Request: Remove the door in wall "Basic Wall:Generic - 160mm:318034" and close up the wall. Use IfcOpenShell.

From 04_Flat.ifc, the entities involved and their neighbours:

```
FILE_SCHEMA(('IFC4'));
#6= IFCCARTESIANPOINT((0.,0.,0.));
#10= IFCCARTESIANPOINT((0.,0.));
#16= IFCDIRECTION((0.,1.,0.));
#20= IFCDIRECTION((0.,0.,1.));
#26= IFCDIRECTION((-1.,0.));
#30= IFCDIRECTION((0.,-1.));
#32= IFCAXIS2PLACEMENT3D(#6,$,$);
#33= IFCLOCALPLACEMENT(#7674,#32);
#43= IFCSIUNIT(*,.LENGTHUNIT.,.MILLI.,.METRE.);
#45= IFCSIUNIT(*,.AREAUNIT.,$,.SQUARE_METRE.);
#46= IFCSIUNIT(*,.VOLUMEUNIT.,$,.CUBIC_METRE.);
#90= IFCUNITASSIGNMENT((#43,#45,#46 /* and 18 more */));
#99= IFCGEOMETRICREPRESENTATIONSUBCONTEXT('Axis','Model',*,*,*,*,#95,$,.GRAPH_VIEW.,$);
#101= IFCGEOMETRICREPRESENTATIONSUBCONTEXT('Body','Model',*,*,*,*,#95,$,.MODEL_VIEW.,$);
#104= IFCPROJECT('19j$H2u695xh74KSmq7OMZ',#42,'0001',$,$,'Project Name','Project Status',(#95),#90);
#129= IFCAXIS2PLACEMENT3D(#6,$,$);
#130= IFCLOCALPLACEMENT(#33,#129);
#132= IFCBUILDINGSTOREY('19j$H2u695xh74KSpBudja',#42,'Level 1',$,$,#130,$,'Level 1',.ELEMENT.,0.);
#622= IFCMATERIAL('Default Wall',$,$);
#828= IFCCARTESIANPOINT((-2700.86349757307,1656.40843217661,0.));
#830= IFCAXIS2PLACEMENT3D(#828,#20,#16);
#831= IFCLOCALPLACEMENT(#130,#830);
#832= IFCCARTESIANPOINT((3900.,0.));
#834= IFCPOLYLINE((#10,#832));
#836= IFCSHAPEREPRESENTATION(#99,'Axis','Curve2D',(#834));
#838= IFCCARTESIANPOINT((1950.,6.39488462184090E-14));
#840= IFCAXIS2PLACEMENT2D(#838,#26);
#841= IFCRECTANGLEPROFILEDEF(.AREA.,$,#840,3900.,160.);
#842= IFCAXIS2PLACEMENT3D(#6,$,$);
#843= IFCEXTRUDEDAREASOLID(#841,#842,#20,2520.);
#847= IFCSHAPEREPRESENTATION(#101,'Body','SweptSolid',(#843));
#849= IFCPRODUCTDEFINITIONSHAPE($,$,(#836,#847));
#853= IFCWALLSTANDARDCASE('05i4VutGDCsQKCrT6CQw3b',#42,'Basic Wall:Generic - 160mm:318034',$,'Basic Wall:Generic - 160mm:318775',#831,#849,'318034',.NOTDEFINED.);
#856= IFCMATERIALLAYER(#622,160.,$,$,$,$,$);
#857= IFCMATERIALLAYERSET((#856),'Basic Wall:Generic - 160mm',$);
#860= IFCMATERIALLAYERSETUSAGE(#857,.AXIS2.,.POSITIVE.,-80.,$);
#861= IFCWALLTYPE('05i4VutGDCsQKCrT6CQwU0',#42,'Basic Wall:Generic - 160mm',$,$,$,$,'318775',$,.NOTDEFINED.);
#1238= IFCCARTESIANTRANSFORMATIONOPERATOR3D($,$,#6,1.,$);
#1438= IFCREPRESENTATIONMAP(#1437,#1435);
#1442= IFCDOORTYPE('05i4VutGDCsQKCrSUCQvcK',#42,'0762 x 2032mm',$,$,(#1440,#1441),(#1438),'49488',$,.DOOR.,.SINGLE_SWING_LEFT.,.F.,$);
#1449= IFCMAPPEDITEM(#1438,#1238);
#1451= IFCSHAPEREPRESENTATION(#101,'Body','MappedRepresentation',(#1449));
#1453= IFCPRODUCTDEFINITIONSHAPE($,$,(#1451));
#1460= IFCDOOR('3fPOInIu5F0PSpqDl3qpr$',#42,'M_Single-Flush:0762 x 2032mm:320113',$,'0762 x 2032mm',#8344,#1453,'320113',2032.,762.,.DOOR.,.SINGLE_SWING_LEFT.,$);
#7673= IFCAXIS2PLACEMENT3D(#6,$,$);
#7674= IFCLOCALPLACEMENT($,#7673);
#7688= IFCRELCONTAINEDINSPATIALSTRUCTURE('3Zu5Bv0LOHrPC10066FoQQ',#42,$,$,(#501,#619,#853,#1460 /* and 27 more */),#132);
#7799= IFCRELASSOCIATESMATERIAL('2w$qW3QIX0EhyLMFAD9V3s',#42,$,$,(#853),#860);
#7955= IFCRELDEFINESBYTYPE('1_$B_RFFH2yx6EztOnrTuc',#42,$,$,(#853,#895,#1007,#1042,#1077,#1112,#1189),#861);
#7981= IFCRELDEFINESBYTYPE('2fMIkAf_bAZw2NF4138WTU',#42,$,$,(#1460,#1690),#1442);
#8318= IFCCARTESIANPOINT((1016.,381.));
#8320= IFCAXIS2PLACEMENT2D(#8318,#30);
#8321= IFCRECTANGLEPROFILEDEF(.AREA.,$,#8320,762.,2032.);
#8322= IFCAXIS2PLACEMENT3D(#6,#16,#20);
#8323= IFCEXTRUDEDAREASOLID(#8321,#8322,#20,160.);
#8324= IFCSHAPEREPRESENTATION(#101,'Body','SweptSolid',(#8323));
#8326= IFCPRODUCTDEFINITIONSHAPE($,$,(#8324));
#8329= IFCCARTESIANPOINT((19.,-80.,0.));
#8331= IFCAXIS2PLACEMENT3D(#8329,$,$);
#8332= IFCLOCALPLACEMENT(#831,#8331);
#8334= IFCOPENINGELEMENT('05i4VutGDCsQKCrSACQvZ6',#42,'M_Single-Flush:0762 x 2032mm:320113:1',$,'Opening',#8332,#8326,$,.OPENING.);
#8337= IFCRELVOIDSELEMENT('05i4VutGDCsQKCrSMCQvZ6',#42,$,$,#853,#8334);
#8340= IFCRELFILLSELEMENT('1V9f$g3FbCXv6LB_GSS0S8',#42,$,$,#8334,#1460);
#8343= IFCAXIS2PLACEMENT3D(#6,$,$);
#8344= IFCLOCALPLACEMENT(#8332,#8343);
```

```python
import ifcopenshell
import ifcopenshell.api.feature
import ifcopenshell.api.root
import ifcopenshell.geom
import ifcopenshell.util.shape

model = ifcopenshell.open("04_Flat.ifc")
settings = ifcopenshell.geom.settings()


def volume(element):
    """Net volume in cubic metres, openings subtracted."""
    shape = ifcopenshell.geom.create_shape(settings, element)
    return ifcopenshell.util.shape.get_volume(shape.geometry)


door = model.by_guid("3fPOInIu5F0PSpqDl3qpr$")
opening = door.FillsVoids[0].RelatingOpeningElement
wall = opening.VoidsElements[0].RelatingBuildingElement
before = volume(wall)

ifcopenshell.api.root.remove_product(model, product=door)
ifcopenshell.api.feature.remove_feature(model, feature=opening)

after = volume(wall)

print(f"wall volume {before:.3f} -> {after:.3f} m3")

model.write("04_Flat_rev.ifc")
```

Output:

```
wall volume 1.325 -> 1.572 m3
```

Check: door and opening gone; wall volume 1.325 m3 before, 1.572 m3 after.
